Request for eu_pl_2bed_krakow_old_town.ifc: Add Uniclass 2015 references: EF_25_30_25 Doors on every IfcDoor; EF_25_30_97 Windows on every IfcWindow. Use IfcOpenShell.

First a look at what the model holds.

```python
import ifcopenshell

model = ifcopenshell.open("eu_pl_2bed_krakow_old_town.ifc")
print(model.schema)
print("classifications:", [c.Name for c in model.by_type("IfcClassification")])
for ifc_class in ("IfcDoor", "IfcRoof", "IfcStair", "IfcWall", "IfcWindow"):
    print(ifc_class, len(model.by_type(ifc_class)))
```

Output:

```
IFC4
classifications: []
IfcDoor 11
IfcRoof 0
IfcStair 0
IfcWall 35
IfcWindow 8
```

```python
import ifcopenshell
import ifcopenshell.api.classification

model = ifcopenshell.open("eu_pl_2bed_krakow_old_town.ifc")

system = ifcopenshell.api.classification.add_classification(model, classification="Uniclass 2015")

codes = {
    "IfcDoor": ("EF_25_30_25", "Doors"),
    "IfcWindow": ("EF_25_30_97", "Windows"),
}
for ifc_class, (code, name) in codes.items():
    products = model.by_type(ifc_class)
    ifcopenshell.api.classification.add_reference(
        model, products=products, classification=system, identification=code, name=name
    )
    print(code, len(products))

model.write("eu_pl_2bed_krakow_old_town_v2.ifc")
```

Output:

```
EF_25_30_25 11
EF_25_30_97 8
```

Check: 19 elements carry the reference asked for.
